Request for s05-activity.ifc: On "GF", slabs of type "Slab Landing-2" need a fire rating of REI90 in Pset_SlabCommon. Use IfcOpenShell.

First a look at what the model holds.

```python
import ifcopenshell
import ifcopenshell.util.element

model = ifcopenshell.open("s05-activity.ifc")
print(model.schema)
storey = next(s for s in model.by_type("IfcBuildingStorey") if s.Name == "GF")
slabs = [e for e in ifcopenshell.util.element.get_decomposition(storey) if e.is_a("IfcSlab")]
seen = {}
for e in slabs:
    element_type = ifcopenshell.util.element.get_type(e)
    key = (element_type.Name if element_type != e and element_type else None, ifcopenshell.util.element.get_pset(e, "Pset_SlabCommon", "FireRating"))
    seen[key] = seen.get(key, 0) + 1
for (name, value), count in sorted(seen.items(), key=str):
    print(count, "x", name, "|", value)
```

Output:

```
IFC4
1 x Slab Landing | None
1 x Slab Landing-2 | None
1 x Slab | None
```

```python
import ifcopenshell
import ifcopenshell.api.pset
import ifcopenshell.util.element

model = ifcopenshell.open("s05-activity.ifc")

storey = next(s for s in model.by_type("IfcBuildingStorey") if s.Name == "GF")
slabs = [e for e in ifcopenshell.util.element.get_decomposition(storey) if e.is_a("IfcSlab")]

count = 0
for e in slabs:
    element_type = ifcopenshell.util.element.get_type(e)
    if element_type in (None, e) or element_type.Name != "Slab Landing-2":
        continue
    # add_pset returns the element's existing set when there is one.
    pset = ifcopenshell.api.pset.add_pset(model, product=e, name="Pset_SlabCommon")
    ifcopenshell.api.pset.edit_pset(model, pset=pset, properties={"FireRating": "REI90"})
    count += 1

print(count, "slabs updated")

model.write("s05-activity-out.ifc")
```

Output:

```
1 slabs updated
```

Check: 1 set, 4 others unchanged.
